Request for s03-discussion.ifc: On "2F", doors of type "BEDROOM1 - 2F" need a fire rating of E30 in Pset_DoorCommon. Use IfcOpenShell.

First a look at what the model holds.

```python
import ifcopenshell
import ifcopenshell.util.element

model = ifcopenshell.open("s03-discussion.ifc")
print(model.schema)
storey = next(s for s in model.by_type("IfcBuildingStorey") if s.Name == "2F")
doors = [e for e in ifcopenshell.util.element.get_decomposition(storey) if e.is_a("IfcDoor")]
seen = {}
for e in doors:
    element_type = ifcopenshell.util.element.get_type(e)
    key = (element_type.Name if element_type != e and element_type else None, ifcopenshell.util.element.get_pset(e, "Pset_DoorCommon", "FireRating"))
    seen[key] = seen.get(key, 0) + 1
for (name, value), count in sorted(seen.items(), key=str):
    print(count, "x", name, "|", value)
```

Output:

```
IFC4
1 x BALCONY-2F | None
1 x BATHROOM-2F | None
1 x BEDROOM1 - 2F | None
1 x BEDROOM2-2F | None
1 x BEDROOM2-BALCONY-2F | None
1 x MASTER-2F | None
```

```python
import ifcopenshell
import ifcopenshell.api.pset
import ifcopenshell.util.element

model = ifcopenshell.open("s03-discussion.ifc")

storey = next(s for s in model.by_type("IfcBuildingStorey") if s.Name == "2F")
doors = [e for e in ifcopenshell.util.element.get_decomposition(storey) if e.is_a("IfcDoor")]

count = 0
for e in doors:
    element_type = ifcopenshell.util.element.get_type(e)
    if element_type in (None, e) or element_type.Name != "BEDROOM1 - 2F":
        continue
    # add_pset returns the element's existing set when there is one.
    pset = ifcopenshell.api.pset.add_pset(model, product=e, name="Pset_DoorCommon")
    ifcopenshell.api.pset.edit_pset(model, pset=pset, properties={"FireRating": "E30"})
    count += 1

print(count, "doors updated")

model.write("s03-discussion_updated.ifc")
```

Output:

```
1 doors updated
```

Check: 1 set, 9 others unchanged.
